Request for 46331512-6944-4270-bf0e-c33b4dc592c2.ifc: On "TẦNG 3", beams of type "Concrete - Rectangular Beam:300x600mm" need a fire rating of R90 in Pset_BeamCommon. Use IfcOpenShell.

First a look at what the model holds.

```python
import ifcopenshell
import ifcopenshell.util.element

model = ifcopenshell.open("46331512-6944-4270-bf0e-c33b4dc592c2.ifc")
print(model.schema)
storey = next(s for s in model.by_type("IfcBuildingStorey") if s.Name == "TẦNG 3")
beams = [e for e in ifcopenshell.util.element.get_decomposition(storey) if e.is_a("IfcBeam")]
seen = {}
for e in beams:
    element_type = ifcopenshell.util.element.get_type(e)
    key = (element_type.Name if element_type != e and element_type else None, ifcopenshell.util.element.get_pset(e, "Pset_BeamCommon", "FireRating"))
    seen[key] = seen.get(key, 0) + 1
for (name, value), count in sorted(seen.items(), key=str):
    print(count, "x", name, "|", value)
```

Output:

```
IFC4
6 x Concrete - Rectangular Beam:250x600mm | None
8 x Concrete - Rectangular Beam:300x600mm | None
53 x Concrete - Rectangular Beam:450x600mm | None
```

```python
import ifcopenshell
import ifcopenshell.api.pset
import ifcopenshell.util.element

model = ifcopenshell.open("46331512-6944-4270-bf0e-c33b4dc592c2.ifc")

storey = next(s for s in model.by_type("IfcBuildingStorey") if s.Name == "TẦNG 3")
beams = [e for e in ifcopenshell.util.element.get_decomposition(storey) if e.is_a("IfcBeam")]

count = 0
for e in beams:
    element_type = ifcopenshell.util.element.get_type(e)
    if element_type in (None, e) or element_type.Name != "Concrete - Rectangular Beam:300x600mm":
        continue
    # add_pset returns the element's existing set when there is one.
    pset = ifcopenshell.api.pset.add_pset(model, product=e, name="Pset_BeamCommon")
    ifcopenshell.api.pset.edit_pset(model, pset=pset, properties={"FireRating": "R90"})
    count += 1

print(count, "beams updated")

model.write("46331512-6944-4270-bf0e-c33b4dc592c2-out.ifc")
```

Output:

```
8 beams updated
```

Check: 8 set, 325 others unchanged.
